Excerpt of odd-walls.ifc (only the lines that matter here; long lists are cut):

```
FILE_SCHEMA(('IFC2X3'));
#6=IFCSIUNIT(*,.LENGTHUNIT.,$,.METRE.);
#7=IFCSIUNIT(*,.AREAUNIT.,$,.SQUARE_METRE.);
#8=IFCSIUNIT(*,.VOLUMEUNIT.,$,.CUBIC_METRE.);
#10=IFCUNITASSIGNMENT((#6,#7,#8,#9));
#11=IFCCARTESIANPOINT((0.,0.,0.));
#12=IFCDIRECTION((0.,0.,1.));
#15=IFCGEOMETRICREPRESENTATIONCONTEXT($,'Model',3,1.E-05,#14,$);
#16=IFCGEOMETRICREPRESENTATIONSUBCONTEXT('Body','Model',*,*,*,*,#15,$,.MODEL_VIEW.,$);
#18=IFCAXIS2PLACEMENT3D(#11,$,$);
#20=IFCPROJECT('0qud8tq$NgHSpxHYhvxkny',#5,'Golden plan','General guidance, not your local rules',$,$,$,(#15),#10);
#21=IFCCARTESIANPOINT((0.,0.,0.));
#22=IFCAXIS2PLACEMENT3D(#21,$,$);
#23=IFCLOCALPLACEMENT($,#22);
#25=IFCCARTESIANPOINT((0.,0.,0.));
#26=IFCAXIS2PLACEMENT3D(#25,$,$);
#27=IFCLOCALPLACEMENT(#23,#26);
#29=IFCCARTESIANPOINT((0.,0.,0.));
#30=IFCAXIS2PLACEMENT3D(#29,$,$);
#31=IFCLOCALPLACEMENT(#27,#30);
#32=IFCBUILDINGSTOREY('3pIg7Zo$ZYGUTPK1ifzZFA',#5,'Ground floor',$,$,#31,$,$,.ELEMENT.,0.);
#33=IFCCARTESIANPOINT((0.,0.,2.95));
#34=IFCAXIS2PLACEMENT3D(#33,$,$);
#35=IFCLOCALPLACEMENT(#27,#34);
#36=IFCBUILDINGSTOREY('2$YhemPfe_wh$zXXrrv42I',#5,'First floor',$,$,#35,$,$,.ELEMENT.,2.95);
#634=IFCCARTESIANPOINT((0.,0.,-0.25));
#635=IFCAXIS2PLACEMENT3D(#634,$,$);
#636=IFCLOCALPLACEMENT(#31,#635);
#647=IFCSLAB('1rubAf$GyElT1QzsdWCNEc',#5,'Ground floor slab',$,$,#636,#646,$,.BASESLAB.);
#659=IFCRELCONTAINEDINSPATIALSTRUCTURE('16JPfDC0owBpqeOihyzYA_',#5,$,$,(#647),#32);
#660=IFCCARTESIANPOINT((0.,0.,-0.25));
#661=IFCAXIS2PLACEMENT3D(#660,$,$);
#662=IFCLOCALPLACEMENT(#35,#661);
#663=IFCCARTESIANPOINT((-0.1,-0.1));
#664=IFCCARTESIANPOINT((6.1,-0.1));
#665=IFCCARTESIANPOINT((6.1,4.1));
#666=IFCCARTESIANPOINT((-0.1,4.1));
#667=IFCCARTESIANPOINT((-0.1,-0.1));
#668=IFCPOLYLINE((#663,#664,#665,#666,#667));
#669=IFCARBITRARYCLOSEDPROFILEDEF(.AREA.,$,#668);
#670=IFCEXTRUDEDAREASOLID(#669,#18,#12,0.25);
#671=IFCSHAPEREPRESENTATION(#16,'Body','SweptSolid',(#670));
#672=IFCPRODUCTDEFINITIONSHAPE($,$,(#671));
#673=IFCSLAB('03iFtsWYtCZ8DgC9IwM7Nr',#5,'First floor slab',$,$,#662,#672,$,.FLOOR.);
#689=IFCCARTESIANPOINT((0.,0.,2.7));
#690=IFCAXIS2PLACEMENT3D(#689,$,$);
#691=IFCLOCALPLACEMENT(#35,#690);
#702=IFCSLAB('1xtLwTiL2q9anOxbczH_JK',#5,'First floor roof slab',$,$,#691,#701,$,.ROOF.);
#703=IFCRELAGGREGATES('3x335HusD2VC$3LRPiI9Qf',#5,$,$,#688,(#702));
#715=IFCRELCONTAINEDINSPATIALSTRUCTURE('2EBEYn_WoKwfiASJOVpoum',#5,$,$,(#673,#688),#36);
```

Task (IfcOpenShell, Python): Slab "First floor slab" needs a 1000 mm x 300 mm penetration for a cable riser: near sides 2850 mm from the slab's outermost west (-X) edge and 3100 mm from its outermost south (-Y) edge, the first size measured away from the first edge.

```python
import numpy as np
import ifcopenshell
import ifcopenshell.api.feature
import ifcopenshell.api.geometry
import ifcopenshell.api.root
import ifcopenshell.geom
import ifcopenshell.util.placement
import ifcopenshell.util.representation
import ifcopenshell.util.shape
import ifcopenshell.util.unit

model = ifcopenshell.open("odd-walls.ifc")
unit_scale = ifcopenshell.util.unit.calculate_unit_scale(model)
settings = ifcopenshell.geom.settings()


def volume(element):
    """Net volume in cubic metres, openings subtracted."""
    shape = ifcopenshell.geom.create_shape(settings, element)
    return ifcopenshell.util.shape.get_volume(shape.geometry)


slab = model.by_id(673)
before = volume(slab)

# Extent in the slab's own axes, in metres. The edges named are its -X and -Y sides.
slab_shape = ifcopenshell.geom.create_shape(settings, slab)
vertices = ifcopenshell.util.shape.get_vertices(slab_shape.geometry)
x_min, y_min, bottom = vertices.min(axis=0)
top = vertices[:, 2].max()

opening = ifcopenshell.api.root.create_entity(model, ifc_class="IfcOpeningElement", name="Cable riser opening")
context = ifcopenshell.util.representation.get_context(model, "Model", "Body", "MODEL_VIEW")
width, depth = 1, 0.3
outline = [(0.0, 0.0), (width, 0.0), (width, depth), (0.0, depth), (0.0, 0.0)]
# Overshoot both faces by 50 mm so the cut is clean.
shape = ifcopenshell.api.geometry.add_slab_representation(
    model, context=context, depth=top - bottom + 0.1, polyline=outline
)
ifcopenshell.api.geometry.assign_representation(model, product=opening, representation=shape)

matrix = ifcopenshell.util.placement.get_local_placement(slab.ObjectPlacement)
matrix[:, 3] = matrix @ np.append(np.array([x_min + 2.85, y_min + 3.1, bottom - 0.05]) / unit_scale, 1.0)
ifcopenshell.api.geometry.edit_object_placement(model, product=opening, matrix=matrix, is_si=False)
ifcopenshell.api.feature.add_feature(model, feature=opening, element=slab)

after = volume(slab)

print(f"slab volume {before:.3f} -> {after:.3f} m3")

model.write("odd-walls-out.ifc")
```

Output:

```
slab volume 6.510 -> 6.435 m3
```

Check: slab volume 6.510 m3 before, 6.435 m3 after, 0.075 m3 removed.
